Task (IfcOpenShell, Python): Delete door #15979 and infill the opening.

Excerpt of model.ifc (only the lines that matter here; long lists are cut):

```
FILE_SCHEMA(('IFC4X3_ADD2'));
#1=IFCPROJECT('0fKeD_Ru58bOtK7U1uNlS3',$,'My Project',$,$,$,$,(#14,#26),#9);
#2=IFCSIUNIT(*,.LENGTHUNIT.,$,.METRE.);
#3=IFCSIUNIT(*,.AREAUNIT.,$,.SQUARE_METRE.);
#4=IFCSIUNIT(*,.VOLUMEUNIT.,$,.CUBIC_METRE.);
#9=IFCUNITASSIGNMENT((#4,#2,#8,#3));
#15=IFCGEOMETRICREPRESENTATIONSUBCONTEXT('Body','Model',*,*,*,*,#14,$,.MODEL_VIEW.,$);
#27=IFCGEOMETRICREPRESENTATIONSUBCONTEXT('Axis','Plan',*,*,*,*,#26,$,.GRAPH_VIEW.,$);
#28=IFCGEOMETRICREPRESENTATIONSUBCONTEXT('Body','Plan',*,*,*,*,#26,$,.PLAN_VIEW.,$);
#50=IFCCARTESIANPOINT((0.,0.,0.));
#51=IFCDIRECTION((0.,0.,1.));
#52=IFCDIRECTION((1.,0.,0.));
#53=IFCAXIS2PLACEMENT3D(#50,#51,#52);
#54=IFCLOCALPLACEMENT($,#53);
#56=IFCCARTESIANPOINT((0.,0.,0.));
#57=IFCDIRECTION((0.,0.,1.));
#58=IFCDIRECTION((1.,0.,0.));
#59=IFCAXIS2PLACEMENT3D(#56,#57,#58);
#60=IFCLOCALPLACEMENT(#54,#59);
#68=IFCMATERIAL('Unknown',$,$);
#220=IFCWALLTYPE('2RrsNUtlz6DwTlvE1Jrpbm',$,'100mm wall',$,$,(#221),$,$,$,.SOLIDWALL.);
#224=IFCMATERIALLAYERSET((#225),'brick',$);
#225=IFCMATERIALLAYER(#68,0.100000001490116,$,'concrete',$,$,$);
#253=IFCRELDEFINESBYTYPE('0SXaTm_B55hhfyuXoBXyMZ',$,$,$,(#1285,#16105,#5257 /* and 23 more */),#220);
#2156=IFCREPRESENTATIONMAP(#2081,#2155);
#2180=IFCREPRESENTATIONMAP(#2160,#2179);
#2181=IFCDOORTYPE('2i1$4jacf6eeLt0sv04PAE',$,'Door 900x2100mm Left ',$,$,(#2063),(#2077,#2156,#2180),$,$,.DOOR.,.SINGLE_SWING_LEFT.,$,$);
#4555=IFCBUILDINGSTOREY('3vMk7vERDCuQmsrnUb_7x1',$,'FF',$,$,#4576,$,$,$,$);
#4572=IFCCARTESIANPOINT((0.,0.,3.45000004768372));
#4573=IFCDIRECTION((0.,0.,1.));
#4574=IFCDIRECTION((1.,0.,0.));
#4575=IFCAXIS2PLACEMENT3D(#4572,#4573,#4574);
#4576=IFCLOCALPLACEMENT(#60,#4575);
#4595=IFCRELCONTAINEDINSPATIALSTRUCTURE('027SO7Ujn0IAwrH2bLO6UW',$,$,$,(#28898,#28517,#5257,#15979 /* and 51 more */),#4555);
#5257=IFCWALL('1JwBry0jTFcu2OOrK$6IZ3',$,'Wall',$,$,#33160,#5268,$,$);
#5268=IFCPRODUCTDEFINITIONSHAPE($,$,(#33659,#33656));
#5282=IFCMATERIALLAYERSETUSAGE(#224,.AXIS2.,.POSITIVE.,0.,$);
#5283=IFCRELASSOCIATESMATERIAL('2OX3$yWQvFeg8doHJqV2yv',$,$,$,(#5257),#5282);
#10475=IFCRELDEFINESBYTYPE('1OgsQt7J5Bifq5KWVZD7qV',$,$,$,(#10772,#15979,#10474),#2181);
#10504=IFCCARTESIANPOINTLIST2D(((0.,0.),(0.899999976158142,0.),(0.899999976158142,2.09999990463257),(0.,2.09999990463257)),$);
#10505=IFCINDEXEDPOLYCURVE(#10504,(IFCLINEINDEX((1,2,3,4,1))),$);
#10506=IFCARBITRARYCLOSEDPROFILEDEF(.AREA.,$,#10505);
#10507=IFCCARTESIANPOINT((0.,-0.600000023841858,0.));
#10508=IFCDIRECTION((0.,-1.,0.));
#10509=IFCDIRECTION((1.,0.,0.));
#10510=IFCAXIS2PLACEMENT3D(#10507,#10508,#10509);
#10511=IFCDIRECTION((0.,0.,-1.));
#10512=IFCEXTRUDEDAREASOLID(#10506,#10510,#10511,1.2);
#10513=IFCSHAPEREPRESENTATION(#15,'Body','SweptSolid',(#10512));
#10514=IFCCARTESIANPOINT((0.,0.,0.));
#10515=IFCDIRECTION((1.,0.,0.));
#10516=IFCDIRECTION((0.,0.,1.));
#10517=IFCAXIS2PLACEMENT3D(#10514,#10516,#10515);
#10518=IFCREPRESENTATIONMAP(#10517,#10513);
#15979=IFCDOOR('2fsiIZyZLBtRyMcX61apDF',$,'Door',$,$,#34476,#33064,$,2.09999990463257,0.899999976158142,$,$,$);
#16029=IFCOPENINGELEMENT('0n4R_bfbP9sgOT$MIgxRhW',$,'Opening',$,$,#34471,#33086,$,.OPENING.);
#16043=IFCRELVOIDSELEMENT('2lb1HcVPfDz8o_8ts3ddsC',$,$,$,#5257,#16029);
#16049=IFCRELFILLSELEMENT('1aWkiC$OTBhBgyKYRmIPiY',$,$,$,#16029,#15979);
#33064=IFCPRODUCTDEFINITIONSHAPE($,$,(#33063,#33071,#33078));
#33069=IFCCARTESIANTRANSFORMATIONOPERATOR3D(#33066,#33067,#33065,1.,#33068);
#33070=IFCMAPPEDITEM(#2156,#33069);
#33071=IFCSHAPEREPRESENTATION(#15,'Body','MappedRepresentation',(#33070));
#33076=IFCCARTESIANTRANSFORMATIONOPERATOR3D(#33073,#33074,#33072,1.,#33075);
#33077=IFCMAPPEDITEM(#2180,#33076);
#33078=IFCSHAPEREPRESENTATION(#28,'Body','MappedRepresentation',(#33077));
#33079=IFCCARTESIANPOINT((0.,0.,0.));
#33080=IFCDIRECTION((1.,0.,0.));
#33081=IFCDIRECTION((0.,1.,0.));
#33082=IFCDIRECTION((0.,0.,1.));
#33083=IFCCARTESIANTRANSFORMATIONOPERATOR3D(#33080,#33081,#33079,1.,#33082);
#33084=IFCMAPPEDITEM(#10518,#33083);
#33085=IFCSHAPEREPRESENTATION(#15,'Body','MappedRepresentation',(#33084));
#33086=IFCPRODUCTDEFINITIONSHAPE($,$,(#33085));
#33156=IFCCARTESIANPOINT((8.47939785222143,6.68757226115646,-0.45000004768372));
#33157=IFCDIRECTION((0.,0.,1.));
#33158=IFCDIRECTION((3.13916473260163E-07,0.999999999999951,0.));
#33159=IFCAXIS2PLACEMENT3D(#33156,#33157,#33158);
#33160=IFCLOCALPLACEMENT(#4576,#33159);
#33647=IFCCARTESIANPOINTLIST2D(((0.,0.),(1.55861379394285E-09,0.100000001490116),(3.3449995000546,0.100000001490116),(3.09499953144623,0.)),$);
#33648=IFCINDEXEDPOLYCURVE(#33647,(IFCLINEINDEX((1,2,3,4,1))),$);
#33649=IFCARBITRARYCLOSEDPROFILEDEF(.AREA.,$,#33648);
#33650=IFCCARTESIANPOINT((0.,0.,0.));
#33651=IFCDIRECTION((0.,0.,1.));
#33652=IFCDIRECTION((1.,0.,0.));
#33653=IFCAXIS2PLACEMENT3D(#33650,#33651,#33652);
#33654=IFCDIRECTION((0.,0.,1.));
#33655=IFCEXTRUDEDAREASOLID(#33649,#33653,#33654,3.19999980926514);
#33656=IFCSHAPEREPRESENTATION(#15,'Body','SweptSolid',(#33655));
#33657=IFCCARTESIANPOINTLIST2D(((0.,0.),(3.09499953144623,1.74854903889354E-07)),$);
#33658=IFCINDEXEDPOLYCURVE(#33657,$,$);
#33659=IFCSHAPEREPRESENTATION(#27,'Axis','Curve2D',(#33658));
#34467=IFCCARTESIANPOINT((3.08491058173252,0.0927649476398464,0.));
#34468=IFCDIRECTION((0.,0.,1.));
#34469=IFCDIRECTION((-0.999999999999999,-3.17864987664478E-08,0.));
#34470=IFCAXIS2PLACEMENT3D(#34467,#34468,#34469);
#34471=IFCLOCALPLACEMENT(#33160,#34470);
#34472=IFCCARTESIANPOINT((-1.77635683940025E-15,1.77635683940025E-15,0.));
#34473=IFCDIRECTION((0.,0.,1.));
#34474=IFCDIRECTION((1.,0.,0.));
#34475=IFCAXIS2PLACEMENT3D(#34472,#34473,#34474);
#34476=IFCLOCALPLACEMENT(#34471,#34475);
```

```python
import ifcopenshell
import ifcopenshell.api.feature
import ifcopenshell.api.root
import ifcopenshell.geom
import ifcopenshell.util.shape

model = ifcopenshell.open("model.ifc")
settings = ifcopenshell.geom.settings()


def volume(element):
    """Net volume in cubic metres, openings subtracted."""
    shape = ifcopenshell.geom.create_shape(settings, element)
    return ifcopenshell.util.shape.get_volume(shape.geometry)


door = model.by_id(15979)
opening = door.FillsVoids[0].RelatingOpeningElement
wall = opening.VoidsElements[0].RelatingBuildingElement
before = volume(wall)

ifcopenshell.api.root.remove_product(model, product=door)
ifcopenshell.api.feature.remove_feature(model, feature=opening)

after = volume(wall)

print(f"wall volume {before:.3f} -> {after:.3f} m3")

model.write("model_edited.ifc")
```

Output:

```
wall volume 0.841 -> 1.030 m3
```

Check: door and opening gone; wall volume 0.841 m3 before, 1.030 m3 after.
